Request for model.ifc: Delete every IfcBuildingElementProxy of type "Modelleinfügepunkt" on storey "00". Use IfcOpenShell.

First a look at what the model holds.

```python
import ifcopenshell
import ifcopenshell.util.element

model = ifcopenshell.open("model.ifc")
print(model.schema)
storey = next(s for s in model.by_type("IfcBuildingStorey") if s.Name == "00")
proxies = [e for e in ifcopenshell.util.element.get_decomposition(storey) if e.is_a("IfcBuildingElementProxy")]
seen = {}
for e in proxies:
    element_type = ifcopenshell.util.element.get_type(e)
    name = element_type.Name if element_type not in (None, e) else None
    seen[name] = seen.get(name, 0) + 1
for name, count in sorted(seen.items(), key=str):
    print(count, "x", name)
```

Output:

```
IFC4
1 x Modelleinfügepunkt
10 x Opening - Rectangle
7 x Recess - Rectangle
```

```python
import ifcopenshell
import ifcopenshell.api.root
import ifcopenshell.util.element

model = ifcopenshell.open("model.ifc")

storey = next(s for s in model.by_type("IfcBuildingStorey") if s.Name == "00")
proxies = [e for e in ifcopenshell.util.element.get_decomposition(storey) if e.is_a("IfcBuildingElementProxy")]
targets = [e for e in proxies if (t := ifcopenshell.util.element.get_type(e)) not in (None, e) and t.Name == "Modelleinfügepunkt"]

for e in targets:
    ifcopenshell.api.root.remove_product(model, product=e)
print(len(targets), "removed")

model.write("model_rev.ifc")
```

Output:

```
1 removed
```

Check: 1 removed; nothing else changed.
